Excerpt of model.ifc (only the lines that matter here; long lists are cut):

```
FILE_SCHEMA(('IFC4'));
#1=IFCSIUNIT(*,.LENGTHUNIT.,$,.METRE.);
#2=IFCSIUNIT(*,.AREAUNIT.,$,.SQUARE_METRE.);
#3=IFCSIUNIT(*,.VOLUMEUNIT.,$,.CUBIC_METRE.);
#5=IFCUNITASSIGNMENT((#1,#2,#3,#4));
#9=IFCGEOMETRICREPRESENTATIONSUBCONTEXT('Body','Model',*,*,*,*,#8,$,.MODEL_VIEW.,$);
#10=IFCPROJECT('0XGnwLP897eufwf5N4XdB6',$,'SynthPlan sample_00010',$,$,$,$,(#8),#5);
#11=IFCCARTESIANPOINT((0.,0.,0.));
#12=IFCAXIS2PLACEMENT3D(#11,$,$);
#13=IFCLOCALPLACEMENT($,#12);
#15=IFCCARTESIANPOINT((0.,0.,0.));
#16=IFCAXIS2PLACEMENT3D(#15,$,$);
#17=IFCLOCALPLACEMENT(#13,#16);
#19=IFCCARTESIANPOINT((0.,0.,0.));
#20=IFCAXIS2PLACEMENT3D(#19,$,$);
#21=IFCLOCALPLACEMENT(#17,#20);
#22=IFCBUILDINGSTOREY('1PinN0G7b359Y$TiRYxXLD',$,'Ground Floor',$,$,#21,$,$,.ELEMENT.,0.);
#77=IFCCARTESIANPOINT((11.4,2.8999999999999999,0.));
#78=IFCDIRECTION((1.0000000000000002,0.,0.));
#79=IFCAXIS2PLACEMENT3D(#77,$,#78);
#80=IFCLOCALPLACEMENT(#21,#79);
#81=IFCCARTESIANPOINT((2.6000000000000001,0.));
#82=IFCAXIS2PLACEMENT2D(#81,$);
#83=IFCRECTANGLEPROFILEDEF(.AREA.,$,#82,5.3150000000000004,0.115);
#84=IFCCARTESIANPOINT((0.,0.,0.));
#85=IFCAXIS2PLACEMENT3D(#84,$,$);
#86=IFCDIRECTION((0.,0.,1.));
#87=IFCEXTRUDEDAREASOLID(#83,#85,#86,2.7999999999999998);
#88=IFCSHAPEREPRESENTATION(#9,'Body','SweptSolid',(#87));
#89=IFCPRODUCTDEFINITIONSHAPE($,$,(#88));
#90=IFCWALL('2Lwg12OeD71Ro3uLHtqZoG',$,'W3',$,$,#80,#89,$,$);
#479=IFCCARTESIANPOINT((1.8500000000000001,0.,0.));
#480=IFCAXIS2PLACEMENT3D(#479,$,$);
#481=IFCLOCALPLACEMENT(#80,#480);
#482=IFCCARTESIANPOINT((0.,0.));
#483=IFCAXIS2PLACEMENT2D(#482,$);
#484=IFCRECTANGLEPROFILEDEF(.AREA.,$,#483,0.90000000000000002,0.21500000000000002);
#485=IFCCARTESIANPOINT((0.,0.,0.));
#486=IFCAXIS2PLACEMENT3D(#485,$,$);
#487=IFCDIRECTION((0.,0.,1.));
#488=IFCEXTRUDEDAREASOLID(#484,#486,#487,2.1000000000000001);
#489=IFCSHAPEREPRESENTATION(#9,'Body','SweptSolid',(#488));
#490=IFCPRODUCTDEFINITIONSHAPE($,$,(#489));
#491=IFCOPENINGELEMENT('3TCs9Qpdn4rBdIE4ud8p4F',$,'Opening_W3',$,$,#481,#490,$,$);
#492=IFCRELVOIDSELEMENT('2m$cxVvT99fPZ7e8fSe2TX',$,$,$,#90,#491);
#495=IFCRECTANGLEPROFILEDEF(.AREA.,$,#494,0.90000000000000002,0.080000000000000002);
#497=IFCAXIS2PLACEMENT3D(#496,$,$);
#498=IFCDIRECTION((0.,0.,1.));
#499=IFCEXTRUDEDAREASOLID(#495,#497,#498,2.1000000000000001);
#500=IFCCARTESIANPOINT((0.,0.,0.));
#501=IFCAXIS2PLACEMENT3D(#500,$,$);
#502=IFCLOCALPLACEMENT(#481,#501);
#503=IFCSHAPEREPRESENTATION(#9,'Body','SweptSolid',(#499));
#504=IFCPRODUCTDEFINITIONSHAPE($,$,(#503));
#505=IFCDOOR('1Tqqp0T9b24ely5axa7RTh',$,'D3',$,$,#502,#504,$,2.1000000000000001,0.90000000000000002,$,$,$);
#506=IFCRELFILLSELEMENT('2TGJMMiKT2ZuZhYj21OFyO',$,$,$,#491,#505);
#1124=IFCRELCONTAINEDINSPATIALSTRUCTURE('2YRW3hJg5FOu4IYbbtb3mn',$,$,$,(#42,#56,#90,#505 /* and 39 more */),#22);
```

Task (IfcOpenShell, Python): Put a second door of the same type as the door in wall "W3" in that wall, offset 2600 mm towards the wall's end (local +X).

```python
import ifcopenshell
import ifcopenshell.api.feature
import ifcopenshell.api.geometry
import ifcopenshell.api.root
import ifcopenshell.geom
import ifcopenshell.util.element
import ifcopenshell.util.placement
import ifcopenshell.util.shape
import ifcopenshell.util.unit

model = ifcopenshell.open("model.ifc")
unit_scale = ifcopenshell.util.unit.calculate_unit_scale(model)
settings = ifcopenshell.geom.settings()


def volume(element):
    """Net volume in cubic metres, openings subtracted."""
    shape = ifcopenshell.geom.create_shape(settings, element)
    return ifcopenshell.util.shape.get_volume(shape.geometry)


door = model.by_guid("1Tqqp0T9b24ely5axa7RTh")
opening = door.FillsVoids[0].RelatingOpeningElement
wall = opening.VoidsElements[0].RelatingBuildingElement
before = volume(wall)
shift = ifcopenshell.util.placement.get_local_placement(wall.ObjectPlacement)[:3, 0] * 2.6 / unit_scale

# copy_class copies the void relationship, type, container and properties, but no geometry.
new_opening = ifcopenshell.api.root.copy_class(model, product=opening)
new_opening.Representation = ifcopenshell.util.element.copy_deep(
    model, opening.Representation, exclude=["IfcGeometricRepresentationContext", "IfcRepresentationMap"]
)
new_door = ifcopenshell.api.root.copy_class(model, product=door)
new_door.Representation = ifcopenshell.util.element.copy_deep(
    model, door.Representation, exclude=["IfcGeometricRepresentationContext", "IfcRepresentationMap"]
)
ifcopenshell.api.feature.add_filling(model, opening=new_opening, element=new_door)

for old, new in ((opening, new_opening), (door, new_door)):
    matrix = ifcopenshell.util.placement.get_local_placement(old.ObjectPlacement)
    matrix[:3, 3] += shift
    ifcopenshell.api.geometry.edit_object_placement(model, product=new, matrix=matrix, is_si=False)

after = volume(wall)

print(f"wall volume {before:.3f} -> {after:.3f} m3")

model.write("model_v2.ifc")
```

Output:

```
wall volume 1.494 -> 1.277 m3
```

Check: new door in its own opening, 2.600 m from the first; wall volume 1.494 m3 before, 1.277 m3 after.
